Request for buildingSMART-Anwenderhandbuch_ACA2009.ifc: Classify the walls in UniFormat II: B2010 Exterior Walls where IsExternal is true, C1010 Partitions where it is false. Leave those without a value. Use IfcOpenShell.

First a look at what the model holds.

```python
import ifcopenshell
import ifcopenshell.util.element

model = ifcopenshell.open("buildingSMART-Anwenderhandbuch_ACA2009.ifc")
print(model.schema)
print("classifications:", [c.Name for c in model.by_type("IfcClassification")])
values = [ifcopenshell.util.element.get_pset(e, "Pset_WallCommon", "IsExternal") for e in model.by_type("IfcWall")]
for value in (True, False, None):
    print("IsExternal", value, values.count(value))
```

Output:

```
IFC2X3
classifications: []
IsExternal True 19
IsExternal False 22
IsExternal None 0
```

```python
import ifcopenshell
import ifcopenshell.api.classification
import ifcopenshell.util.element

model = ifcopenshell.open("buildingSMART-Anwenderhandbuch_ACA2009.ifc")

# IFC2X3 requires Source and Edition and has no link from the project to the system.
system = model.create_entity("IfcClassification", Source="ASTM", Edition="E1557", Name="UniFormat II")

walls = model.by_type("IfcWall")
external = {e: ifcopenshell.util.element.get_pset(e, "Pset_WallCommon", "IsExternal") for e in walls}
for flag, code, name in ((True, "B2010", "Exterior Walls"), (False, "C1010", "Partitions")):
    products = [e for e in walls if external[e] is flag]
    ifcopenshell.api.classification.add_reference(
        model, products=products, classification=system, identification=code, name=name
    )
    print(code, len(products))

model.write("buildingSMART-Anwenderhandbuch_ACA2009-out.ifc")
```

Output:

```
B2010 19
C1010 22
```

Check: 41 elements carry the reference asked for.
